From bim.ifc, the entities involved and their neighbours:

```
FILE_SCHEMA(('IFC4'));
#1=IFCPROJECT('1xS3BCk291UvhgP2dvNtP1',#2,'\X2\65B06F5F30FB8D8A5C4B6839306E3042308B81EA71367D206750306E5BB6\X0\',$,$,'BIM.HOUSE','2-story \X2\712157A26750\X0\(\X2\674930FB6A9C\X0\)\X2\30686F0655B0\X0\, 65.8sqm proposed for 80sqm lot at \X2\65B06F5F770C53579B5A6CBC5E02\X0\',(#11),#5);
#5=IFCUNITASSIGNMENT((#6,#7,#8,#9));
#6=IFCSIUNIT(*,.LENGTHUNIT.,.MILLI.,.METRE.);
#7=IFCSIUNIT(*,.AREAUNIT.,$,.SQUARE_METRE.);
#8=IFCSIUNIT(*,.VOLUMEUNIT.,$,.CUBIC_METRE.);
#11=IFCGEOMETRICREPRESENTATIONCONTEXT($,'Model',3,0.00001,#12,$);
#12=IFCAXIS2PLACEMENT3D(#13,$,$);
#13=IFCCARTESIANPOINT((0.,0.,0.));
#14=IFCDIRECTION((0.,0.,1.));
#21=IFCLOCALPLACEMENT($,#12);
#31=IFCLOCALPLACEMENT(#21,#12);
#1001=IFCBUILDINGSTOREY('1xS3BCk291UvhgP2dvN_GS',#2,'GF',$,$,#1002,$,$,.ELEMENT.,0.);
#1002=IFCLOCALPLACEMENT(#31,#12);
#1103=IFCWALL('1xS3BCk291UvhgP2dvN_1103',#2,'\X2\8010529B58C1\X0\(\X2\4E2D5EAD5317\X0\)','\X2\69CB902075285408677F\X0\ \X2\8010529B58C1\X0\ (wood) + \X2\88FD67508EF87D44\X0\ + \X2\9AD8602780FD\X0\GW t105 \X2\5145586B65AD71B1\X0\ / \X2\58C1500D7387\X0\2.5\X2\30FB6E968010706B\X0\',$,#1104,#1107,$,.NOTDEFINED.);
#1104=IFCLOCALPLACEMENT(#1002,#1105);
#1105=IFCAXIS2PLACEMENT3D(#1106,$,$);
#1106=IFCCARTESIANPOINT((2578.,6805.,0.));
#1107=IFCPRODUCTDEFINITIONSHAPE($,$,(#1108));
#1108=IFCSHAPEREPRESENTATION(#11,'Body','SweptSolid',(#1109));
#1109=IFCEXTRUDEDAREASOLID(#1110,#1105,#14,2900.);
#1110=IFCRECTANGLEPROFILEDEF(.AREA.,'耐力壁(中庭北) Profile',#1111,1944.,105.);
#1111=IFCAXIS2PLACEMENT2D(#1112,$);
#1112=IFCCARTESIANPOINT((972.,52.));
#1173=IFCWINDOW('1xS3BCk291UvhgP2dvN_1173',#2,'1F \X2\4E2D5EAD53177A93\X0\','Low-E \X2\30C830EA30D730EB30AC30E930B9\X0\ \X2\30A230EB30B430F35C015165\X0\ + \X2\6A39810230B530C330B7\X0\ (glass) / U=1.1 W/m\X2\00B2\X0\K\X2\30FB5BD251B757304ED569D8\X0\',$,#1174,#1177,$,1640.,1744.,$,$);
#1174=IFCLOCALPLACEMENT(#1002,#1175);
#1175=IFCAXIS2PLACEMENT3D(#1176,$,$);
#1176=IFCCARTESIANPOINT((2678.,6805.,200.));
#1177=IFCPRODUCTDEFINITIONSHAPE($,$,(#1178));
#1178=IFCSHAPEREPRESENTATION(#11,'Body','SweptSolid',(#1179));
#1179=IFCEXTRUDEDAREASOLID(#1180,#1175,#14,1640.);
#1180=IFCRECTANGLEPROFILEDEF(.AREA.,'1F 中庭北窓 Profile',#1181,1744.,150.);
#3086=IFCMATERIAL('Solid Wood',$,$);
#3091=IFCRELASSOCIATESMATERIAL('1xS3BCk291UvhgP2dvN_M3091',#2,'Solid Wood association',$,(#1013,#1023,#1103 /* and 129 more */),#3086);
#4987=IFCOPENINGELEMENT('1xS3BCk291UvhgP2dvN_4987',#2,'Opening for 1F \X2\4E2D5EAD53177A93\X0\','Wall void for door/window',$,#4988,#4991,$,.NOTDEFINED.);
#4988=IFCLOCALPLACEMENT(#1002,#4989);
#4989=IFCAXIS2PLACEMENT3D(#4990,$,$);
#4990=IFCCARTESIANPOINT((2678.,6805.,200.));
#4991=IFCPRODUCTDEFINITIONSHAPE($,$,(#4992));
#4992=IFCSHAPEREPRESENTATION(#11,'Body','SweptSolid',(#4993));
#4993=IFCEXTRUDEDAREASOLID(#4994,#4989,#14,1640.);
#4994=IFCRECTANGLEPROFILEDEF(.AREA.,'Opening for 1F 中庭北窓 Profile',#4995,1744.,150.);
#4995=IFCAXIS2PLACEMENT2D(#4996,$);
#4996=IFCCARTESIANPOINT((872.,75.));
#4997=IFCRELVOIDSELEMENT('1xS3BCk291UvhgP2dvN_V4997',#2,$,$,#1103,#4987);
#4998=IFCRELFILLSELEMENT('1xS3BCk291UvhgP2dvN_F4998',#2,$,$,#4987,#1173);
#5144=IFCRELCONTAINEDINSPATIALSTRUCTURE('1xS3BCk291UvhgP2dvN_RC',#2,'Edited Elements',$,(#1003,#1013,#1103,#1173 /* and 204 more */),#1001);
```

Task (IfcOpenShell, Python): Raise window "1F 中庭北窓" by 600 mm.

```python
import numpy as np
import ifcopenshell
import ifcopenshell.api.geometry
import ifcopenshell.util.placement
import ifcopenshell.util.unit

model = ifcopenshell.open("bim.ifc")
unit_scale = ifcopenshell.util.unit.calculate_unit_scale(model)

window = model.by_id(1173)
opening = window.FillsVoids[0].RelatingOpeningElement
dz = 600.0

shift = np.array([0.0, 0.0, dz])
# The window is not placed relative to its opening, so move both.
for product in (opening, window):
    matrix = ifcopenshell.util.placement.get_local_placement(product.ObjectPlacement)
    matrix[:3, 3] += shift
    ifcopenshell.api.geometry.edit_object_placement(model, product=product, matrix=matrix, is_si=False)

print(f"moved by {dz * unit_scale:+.3f} m")

model.write("bim_edited.ifc")
```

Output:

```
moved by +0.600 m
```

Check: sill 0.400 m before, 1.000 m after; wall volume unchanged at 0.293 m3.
